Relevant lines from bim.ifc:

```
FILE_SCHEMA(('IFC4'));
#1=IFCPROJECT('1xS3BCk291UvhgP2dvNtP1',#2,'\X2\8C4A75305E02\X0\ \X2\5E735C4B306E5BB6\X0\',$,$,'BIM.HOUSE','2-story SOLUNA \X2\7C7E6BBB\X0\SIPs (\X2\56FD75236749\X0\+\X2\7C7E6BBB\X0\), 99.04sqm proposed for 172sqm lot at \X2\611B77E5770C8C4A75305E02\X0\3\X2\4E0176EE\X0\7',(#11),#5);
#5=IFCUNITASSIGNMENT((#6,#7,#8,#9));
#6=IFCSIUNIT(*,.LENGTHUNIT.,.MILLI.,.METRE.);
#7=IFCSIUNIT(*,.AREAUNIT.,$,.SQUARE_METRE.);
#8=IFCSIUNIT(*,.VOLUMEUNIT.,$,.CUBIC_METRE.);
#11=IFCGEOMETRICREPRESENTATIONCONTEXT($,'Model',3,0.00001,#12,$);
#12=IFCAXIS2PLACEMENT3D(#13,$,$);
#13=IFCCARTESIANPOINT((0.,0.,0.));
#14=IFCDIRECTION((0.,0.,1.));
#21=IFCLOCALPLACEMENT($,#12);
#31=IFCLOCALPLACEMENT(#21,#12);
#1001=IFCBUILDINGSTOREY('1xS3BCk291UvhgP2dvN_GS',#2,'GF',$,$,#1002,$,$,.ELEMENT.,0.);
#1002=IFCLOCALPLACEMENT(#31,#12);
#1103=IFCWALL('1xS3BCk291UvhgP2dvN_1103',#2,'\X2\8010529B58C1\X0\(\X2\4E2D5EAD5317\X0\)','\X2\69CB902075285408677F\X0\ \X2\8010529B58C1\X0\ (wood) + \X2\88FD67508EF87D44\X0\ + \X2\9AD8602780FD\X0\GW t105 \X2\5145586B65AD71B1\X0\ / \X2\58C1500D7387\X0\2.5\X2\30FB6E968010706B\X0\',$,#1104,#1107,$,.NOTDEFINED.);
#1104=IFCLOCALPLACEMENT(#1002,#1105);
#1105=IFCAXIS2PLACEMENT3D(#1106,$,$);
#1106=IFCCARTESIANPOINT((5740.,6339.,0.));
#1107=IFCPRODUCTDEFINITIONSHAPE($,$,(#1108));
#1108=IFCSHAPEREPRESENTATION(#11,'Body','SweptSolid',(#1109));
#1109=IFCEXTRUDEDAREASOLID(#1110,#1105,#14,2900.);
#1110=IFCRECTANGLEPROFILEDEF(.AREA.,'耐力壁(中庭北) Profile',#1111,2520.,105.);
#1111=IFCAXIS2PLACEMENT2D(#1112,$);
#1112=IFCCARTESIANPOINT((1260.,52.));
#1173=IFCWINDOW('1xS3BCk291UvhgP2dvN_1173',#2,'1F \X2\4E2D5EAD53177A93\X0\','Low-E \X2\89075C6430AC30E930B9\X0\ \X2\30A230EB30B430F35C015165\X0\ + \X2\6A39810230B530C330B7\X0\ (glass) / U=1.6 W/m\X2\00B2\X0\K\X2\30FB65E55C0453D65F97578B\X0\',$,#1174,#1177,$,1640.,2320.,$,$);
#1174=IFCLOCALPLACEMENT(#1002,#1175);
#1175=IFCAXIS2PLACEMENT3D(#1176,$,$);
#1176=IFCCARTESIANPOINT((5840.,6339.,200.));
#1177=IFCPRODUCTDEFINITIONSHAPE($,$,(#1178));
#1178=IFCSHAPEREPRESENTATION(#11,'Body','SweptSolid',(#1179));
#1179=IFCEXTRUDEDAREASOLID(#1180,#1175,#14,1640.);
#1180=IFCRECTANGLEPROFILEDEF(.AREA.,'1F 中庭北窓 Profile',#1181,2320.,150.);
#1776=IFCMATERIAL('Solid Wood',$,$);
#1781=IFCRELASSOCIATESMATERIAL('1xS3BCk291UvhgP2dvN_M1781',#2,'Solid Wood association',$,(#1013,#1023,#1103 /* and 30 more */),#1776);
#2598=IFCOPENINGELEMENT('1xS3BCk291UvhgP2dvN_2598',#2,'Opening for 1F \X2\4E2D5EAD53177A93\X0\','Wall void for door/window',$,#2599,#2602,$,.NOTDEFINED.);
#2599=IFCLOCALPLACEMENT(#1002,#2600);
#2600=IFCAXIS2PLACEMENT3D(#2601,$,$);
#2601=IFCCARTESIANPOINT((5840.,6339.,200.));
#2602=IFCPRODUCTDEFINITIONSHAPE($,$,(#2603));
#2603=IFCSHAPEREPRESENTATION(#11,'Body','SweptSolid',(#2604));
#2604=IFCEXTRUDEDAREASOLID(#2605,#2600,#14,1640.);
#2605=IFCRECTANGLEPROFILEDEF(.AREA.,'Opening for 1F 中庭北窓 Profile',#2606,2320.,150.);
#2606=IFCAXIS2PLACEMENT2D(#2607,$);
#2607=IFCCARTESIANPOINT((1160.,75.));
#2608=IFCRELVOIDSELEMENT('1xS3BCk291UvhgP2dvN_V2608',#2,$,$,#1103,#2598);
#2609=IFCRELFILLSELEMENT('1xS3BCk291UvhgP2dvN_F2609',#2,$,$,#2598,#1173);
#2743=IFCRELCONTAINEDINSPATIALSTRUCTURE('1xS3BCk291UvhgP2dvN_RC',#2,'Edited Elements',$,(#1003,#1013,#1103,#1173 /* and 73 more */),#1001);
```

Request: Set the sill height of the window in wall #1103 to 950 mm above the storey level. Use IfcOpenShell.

```python
import numpy as np
import ifcopenshell
import ifcopenshell.api.geometry
import ifcopenshell.geom
import ifcopenshell.util.element
import ifcopenshell.util.placement
import ifcopenshell.util.shape
import ifcopenshell.util.unit

model = ifcopenshell.open("bim.ifc")
unit_scale = ifcopenshell.util.unit.calculate_unit_scale(model)

window = model.by_id(1173)
opening = window.FillsVoids[0].RelatingOpeningElement
storey = ifcopenshell.util.element.get_container(window, ifc_class="IfcBuildingStorey")
level = ifcopenshell.util.placement.get_local_placement(storey.ObjectPlacement)[2, 3]

# The opening's origin need not be at the sill, so measure its lowest point.
shape = ifcopenshell.geom.create_shape(ifcopenshell.geom.settings(), opening)
bottom = ifcopenshell.util.shape.get_shape_bottom_elevation(shape, shape.geometry) / unit_scale
dz = level + 0.95 / unit_scale - bottom

shift = np.array([0.0, 0.0, dz])
# The window is not placed relative to its opening, so move both.
for product in (opening, window):
    matrix = ifcopenshell.util.placement.get_local_placement(product.ObjectPlacement)
    matrix[:3, 3] += shift
    ifcopenshell.api.geometry.edit_object_placement(model, product=product, matrix=matrix, is_si=False)

print(f"moved by {dz * unit_scale:+.3f} m")

model.write("bim_v2.ifc")
```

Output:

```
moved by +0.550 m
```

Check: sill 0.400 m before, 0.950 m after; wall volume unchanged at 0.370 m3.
